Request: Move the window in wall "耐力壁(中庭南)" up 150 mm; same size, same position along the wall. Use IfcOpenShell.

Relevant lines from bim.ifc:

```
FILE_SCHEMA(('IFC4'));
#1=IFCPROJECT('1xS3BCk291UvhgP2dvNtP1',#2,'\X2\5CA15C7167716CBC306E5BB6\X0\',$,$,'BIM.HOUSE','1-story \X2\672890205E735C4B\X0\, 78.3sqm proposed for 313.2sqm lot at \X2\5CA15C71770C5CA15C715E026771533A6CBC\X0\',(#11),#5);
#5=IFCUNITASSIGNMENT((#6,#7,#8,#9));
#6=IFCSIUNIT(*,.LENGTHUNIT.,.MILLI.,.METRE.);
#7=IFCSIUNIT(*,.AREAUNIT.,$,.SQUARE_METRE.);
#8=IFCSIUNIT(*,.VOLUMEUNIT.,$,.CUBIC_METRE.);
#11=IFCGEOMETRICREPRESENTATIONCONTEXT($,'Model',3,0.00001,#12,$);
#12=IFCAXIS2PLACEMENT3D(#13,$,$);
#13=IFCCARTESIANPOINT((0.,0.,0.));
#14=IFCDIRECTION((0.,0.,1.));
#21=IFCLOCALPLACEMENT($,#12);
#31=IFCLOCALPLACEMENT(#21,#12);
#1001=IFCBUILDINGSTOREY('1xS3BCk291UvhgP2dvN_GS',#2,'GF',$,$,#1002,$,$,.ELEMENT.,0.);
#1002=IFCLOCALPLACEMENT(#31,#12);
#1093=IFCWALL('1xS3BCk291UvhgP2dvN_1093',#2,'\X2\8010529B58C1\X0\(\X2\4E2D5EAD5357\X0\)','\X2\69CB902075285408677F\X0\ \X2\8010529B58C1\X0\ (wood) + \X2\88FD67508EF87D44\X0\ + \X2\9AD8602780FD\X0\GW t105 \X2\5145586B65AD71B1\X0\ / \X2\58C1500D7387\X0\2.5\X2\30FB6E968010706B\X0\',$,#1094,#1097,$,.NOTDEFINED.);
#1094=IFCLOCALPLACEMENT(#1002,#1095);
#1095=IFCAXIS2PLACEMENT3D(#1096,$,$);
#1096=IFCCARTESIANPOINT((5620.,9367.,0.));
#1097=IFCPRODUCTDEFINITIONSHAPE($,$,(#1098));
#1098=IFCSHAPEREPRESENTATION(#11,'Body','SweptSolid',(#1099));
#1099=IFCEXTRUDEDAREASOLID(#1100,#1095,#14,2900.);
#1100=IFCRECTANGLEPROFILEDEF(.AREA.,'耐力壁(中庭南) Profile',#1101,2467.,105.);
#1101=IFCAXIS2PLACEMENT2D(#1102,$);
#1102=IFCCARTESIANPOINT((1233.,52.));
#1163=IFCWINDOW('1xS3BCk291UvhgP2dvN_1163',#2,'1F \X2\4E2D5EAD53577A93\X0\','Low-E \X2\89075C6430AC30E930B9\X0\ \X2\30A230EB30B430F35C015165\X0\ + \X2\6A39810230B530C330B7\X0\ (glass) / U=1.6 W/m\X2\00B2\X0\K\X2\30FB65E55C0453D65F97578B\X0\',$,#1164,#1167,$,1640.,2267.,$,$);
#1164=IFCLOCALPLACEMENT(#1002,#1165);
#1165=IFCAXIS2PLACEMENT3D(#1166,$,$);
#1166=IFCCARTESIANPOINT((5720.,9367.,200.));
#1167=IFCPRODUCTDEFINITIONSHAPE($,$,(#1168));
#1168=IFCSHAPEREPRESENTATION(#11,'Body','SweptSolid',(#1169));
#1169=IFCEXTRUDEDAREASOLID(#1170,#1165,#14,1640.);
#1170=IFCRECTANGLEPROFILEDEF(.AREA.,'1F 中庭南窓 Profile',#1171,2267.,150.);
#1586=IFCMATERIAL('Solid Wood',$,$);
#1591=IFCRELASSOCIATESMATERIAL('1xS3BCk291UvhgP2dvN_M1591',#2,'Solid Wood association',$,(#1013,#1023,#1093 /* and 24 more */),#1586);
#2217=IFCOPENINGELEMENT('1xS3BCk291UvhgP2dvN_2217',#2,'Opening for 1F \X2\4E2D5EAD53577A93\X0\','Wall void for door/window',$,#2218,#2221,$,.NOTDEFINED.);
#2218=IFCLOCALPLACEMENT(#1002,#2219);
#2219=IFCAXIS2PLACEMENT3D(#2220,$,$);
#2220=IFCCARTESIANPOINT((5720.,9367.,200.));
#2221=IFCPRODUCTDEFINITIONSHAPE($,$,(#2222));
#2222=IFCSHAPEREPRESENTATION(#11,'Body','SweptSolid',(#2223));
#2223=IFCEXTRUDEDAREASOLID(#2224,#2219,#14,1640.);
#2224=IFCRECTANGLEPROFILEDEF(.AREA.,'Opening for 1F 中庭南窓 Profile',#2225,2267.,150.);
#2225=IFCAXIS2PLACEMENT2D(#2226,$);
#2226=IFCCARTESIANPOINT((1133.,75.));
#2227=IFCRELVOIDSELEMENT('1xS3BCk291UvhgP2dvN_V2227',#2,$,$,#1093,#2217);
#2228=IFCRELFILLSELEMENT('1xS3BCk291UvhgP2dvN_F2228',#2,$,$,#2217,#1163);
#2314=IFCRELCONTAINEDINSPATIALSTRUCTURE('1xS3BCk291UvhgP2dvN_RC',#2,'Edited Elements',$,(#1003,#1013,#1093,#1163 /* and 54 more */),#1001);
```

```python
import numpy as np
import ifcopenshell
import ifcopenshell.api.geometry
import ifcopenshell.util.placement
import ifcopenshell.util.unit

model = ifcopenshell.open("bim.ifc")
unit_scale = ifcopenshell.util.unit.calculate_unit_scale(model)

window = model.by_id(1163)
opening = window.FillsVoids[0].RelatingOpeningElement
dz = 0.15 / unit_scale

shift = np.array([0.0, 0.0, dz])
# The window is not placed relative to its opening, so move both.
for product in (opening, window):
    matrix = ifcopenshell.util.placement.get_local_placement(product.ObjectPlacement)
    matrix[:3, 3] += shift
    ifcopenshell.api.geometry.edit_object_placement(model, product=product, matrix=matrix, is_si=False)

print(f"moved by {dz * unit_scale:+.3f} m")

model.write("bim_v2.ifc")
```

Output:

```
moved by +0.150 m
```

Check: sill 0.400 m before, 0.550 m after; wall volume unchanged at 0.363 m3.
